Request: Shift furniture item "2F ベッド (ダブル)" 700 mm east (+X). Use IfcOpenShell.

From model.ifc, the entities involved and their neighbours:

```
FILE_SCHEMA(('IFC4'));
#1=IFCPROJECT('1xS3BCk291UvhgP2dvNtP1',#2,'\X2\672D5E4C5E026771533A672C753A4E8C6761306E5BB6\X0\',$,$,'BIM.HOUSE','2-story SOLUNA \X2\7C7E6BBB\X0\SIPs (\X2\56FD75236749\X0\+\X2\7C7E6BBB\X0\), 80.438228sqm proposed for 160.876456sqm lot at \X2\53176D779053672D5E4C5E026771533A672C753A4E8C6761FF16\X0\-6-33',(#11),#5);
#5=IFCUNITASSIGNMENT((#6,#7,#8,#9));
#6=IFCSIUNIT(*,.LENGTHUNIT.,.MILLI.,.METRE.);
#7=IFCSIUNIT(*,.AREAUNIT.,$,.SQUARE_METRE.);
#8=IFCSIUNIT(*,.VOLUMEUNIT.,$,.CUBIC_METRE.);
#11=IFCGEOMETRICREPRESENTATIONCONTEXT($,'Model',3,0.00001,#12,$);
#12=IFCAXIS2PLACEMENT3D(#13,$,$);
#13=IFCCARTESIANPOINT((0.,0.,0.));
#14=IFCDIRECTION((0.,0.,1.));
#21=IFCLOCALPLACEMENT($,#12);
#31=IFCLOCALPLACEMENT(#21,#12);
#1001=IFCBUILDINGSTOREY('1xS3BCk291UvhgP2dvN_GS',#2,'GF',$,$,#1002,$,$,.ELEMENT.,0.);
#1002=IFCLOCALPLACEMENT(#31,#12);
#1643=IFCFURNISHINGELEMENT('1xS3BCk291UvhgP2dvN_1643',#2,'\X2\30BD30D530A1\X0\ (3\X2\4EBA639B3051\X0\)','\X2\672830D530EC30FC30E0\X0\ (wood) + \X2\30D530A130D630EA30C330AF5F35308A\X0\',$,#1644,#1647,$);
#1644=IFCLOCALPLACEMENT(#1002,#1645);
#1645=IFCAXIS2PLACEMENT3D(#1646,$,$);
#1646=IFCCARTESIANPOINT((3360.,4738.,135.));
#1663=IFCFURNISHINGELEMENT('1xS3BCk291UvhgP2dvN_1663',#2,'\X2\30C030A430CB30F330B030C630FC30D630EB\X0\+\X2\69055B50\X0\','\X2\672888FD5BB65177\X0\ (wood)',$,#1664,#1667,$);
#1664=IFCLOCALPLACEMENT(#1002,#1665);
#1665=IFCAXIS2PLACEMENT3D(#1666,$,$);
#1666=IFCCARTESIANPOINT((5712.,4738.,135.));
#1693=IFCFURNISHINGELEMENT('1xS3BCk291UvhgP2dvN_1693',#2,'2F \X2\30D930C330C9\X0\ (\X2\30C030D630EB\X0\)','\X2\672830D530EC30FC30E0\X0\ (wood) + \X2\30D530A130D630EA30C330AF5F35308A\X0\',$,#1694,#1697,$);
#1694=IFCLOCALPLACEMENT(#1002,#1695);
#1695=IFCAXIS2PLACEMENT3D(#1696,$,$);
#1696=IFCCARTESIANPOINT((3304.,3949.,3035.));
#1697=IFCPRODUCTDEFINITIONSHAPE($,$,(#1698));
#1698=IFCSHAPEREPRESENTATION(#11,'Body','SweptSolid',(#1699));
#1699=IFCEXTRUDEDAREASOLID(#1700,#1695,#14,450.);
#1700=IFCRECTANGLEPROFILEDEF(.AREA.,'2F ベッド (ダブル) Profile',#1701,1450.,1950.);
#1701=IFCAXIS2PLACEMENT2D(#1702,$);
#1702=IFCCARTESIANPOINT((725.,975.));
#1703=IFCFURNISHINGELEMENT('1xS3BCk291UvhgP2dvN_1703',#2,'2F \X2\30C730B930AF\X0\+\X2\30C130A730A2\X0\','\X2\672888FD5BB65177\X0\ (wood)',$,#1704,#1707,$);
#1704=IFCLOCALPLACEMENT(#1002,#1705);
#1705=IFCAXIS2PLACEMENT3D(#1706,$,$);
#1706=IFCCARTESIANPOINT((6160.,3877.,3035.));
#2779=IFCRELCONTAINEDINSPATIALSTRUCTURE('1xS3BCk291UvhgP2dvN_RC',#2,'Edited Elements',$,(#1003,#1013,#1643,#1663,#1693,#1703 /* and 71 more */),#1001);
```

```python
import ifcopenshell
import ifcopenshell.api.geometry
import ifcopenshell.util.placement

model = ifcopenshell.open("model.ifc")

item = model.by_guid("1xS3BCk291UvhgP2dvN_1693")
matrix = ifcopenshell.util.placement.get_local_placement(item.ObjectPlacement)
matrix[0, 3] += 700.0
ifcopenshell.api.geometry.edit_object_placement(model, product=item, matrix=matrix, is_si=False)

print(ifcopenshell.util.placement.get_local_placement(item.ObjectPlacement).round(3) + 0.0)

model.write("model-out.ifc")
```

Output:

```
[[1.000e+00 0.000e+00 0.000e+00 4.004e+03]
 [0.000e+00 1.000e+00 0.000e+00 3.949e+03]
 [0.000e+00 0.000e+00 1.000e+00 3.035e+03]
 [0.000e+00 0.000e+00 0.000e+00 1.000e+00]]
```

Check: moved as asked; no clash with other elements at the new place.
